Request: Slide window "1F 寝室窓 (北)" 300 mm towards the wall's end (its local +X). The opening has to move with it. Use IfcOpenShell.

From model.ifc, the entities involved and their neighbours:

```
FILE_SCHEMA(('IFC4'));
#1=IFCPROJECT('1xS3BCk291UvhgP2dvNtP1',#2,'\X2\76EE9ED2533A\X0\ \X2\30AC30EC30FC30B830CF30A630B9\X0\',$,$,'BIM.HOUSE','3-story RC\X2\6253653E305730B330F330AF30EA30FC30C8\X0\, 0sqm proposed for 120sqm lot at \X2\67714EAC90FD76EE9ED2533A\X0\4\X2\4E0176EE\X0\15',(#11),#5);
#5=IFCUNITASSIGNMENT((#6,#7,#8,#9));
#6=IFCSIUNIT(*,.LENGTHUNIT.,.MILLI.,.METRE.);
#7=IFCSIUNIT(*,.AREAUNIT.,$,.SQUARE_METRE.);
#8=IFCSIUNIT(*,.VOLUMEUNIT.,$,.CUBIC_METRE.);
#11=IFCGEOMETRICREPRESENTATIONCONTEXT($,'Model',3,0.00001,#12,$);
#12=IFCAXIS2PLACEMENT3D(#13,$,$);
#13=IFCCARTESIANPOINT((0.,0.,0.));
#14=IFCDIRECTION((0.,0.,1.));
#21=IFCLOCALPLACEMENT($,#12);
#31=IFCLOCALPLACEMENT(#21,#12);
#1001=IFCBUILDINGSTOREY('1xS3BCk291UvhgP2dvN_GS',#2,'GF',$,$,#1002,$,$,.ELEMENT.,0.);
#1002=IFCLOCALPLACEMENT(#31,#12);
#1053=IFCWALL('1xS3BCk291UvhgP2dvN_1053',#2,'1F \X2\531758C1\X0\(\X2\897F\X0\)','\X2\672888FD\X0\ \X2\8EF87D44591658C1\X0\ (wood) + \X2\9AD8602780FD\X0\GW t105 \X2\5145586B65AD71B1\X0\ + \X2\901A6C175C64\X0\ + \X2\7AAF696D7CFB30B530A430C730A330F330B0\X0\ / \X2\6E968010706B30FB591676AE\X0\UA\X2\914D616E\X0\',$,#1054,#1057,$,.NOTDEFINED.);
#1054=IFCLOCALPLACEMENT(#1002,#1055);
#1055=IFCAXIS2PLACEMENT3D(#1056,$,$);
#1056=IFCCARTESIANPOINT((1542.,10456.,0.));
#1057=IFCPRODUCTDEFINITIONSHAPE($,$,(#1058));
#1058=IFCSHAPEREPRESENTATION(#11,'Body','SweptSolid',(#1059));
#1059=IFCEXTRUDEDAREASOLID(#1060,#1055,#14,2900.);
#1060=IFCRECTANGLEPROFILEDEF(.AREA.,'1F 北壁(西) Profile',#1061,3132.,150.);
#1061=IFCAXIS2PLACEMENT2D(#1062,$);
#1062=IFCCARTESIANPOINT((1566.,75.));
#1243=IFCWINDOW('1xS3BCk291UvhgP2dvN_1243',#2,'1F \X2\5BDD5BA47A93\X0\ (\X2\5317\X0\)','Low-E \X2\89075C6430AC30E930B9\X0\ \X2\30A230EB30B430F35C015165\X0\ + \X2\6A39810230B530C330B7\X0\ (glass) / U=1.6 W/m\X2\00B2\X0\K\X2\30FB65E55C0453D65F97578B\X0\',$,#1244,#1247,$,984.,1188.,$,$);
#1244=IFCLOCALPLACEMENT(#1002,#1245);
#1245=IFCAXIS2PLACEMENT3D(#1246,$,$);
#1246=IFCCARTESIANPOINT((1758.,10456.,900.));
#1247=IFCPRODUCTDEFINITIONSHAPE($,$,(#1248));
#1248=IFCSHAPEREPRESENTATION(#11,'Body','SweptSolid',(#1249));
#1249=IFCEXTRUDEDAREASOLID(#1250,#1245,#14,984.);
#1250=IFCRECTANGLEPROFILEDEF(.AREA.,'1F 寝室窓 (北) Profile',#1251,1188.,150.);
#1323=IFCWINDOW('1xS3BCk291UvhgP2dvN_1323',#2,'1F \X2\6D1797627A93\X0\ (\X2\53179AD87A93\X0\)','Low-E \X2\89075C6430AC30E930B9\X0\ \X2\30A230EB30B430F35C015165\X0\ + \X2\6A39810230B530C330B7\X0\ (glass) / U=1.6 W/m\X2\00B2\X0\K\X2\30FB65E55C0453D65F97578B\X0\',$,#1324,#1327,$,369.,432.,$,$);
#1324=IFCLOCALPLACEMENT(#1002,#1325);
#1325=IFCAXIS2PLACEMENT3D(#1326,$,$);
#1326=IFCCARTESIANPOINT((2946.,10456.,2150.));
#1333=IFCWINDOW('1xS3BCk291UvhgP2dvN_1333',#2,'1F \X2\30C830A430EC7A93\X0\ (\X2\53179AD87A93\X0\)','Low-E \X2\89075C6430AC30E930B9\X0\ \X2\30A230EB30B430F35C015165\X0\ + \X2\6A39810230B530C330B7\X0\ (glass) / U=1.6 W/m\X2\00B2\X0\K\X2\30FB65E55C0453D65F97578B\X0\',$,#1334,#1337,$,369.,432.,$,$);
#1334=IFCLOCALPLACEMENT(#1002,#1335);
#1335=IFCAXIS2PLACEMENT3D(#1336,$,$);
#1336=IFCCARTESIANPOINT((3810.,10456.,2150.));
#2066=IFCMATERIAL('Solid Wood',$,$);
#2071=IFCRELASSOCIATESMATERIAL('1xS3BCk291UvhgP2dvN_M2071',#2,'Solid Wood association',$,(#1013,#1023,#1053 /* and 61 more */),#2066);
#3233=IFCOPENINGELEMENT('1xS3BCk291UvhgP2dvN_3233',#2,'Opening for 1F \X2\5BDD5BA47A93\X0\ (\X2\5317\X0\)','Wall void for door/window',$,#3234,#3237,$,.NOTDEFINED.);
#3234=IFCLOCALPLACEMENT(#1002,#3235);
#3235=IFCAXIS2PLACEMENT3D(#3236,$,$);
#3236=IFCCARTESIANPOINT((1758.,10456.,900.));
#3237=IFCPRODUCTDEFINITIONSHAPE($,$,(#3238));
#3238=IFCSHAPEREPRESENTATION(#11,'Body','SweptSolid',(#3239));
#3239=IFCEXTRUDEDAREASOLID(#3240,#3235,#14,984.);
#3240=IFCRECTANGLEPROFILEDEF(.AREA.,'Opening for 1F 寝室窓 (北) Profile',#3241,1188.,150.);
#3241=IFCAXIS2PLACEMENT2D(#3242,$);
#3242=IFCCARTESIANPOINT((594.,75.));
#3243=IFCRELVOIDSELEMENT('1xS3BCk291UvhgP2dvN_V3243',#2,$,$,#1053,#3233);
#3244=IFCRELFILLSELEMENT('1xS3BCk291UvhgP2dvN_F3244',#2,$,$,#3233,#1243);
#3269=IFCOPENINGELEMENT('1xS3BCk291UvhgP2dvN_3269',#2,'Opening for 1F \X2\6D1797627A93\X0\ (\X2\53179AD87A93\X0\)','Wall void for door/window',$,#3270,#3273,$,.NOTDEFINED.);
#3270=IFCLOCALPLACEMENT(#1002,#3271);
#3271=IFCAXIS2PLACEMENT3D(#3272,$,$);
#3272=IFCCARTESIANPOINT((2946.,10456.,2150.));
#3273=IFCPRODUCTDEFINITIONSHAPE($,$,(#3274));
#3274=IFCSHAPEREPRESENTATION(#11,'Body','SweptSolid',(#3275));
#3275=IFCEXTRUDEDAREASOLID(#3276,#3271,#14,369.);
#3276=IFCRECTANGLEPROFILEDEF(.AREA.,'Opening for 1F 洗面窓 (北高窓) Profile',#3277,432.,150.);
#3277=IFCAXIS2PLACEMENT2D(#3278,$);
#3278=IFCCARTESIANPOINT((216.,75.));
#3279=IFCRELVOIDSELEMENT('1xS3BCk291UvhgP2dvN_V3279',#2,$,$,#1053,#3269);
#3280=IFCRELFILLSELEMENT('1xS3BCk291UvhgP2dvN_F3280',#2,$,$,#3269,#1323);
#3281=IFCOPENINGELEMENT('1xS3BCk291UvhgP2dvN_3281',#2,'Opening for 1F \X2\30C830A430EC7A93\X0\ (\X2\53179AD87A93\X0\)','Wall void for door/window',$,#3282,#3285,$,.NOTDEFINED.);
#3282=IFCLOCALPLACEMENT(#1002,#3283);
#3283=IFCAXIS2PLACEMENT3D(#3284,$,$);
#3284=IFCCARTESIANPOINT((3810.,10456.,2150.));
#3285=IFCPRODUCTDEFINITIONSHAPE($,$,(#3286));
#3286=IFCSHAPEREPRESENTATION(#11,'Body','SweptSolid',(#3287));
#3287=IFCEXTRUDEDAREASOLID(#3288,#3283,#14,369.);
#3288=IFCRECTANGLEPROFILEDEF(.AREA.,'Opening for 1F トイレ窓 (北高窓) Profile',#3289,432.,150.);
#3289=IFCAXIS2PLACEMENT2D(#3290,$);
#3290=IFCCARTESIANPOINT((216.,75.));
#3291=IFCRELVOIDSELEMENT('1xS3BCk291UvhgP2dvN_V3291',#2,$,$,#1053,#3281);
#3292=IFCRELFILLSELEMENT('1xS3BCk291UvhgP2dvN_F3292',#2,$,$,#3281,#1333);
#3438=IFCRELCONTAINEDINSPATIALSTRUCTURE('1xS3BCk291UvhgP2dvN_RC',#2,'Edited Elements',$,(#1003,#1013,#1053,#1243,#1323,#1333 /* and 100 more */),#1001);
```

```python
import ifcopenshell
import ifcopenshell.api.geometry
import ifcopenshell.util.placement
import ifcopenshell.util.unit

model = ifcopenshell.open("model.ifc")
unit_scale = ifcopenshell.util.unit.calculate_unit_scale(model)

window = model.by_guid("1xS3BCk291UvhgP2dvN_1243")
opening = window.FillsVoids[0].RelatingOpeningElement
wall = opening.VoidsElements[0].RelatingBuildingElement

wall_matrix = ifcopenshell.util.placement.get_local_placement(wall.ObjectPlacement)
shift = wall_matrix[:3, 0] * 0.3 / unit_scale
before = ifcopenshell.util.placement.get_local_placement(window.ObjectPlacement)[:3, 3].copy()

# The window is not placed relative to its opening, so move both.
for product in (opening, window):
    matrix = ifcopenshell.util.placement.get_local_placement(product.ObjectPlacement)
    matrix[:3, 3] += shift
    ifcopenshell.api.geometry.edit_object_placement(model, product=product, matrix=matrix, is_si=False)

after = ifcopenshell.util.placement.get_local_placement(window.ObjectPlacement)[:3, 3]
print("window moved by", (after - before).round(3) + 0.0)

model.write("model_rev.ifc")
```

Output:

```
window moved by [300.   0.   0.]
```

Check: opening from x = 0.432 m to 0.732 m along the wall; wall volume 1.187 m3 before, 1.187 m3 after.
